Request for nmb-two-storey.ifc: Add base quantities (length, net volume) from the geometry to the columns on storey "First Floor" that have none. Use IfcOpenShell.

First a look at what the model holds.

```python
import ifcopenshell
import ifcopenshell.util.element
import ifcopenshell.util.unit

model = ifcopenshell.open("nmb-two-storey.ifc")
print(model.schema)
for unit_type in ("LENGTHUNIT", "AREAUNIT", "VOLUMEUNIT"):
    print(unit_type, ifcopenshell.util.unit.calculate_unit_scale(model, unit_type))
storey = next(s for s in model.by_type("IfcBuildingStorey") if s.Name == "First Floor")
columns = [e for e in ifcopenshell.util.element.get_decomposition(storey) if e.is_a("IfcColumn")]
for e in sorted(columns, key=lambda e: e.id()):
    print(e.id(), e.is_a(), e.Name, list(ifcopenshell.util.element.get_psets(e, qtos_only=True)), sep=" | ")
```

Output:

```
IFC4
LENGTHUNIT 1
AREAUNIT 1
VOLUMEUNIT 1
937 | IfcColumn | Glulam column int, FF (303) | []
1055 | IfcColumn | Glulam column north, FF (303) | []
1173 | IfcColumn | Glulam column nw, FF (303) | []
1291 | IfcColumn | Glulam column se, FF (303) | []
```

```python
import ifcopenshell
import ifcopenshell.api.pset
import ifcopenshell.geom
import ifcopenshell.util.element
import ifcopenshell.util.shape
import ifcopenshell.util.unit

model = ifcopenshell.open("nmb-two-storey.ifc")
unit_scale = ifcopenshell.util.unit.calculate_unit_scale(model)
volume_scale = ifcopenshell.util.unit.calculate_unit_scale(model, "VOLUMEUNIT")
settings = ifcopenshell.geom.settings()

storey = next(s for s in model.by_type("IfcBuildingStorey") if s.Name == "First Floor")
columns = [e for e in ifcopenshell.util.element.get_decomposition(storey) if e.is_a("IfcColumn")]

for e in sorted(columns, key=lambda e: e.id()):
    if ifcopenshell.util.element.get_psets(e, qtos_only=True, should_inherit=False):
        continue
    # Geometry comes back in metres, in the element's own axes.
    shape = ifcopenshell.geom.create_shape(settings, e)
    values = {
        "Length": ifcopenshell.util.shape.get_z(shape.geometry) / unit_scale,
        "NetVolume": ifcopenshell.util.shape.get_volume(shape.geometry) / volume_scale,
    }
    qto = ifcopenshell.api.pset.add_qto(model, product=e, name="Qto_ColumnBaseQuantities")
    ifcopenshell.api.pset.edit_qto(model, qto=qto, properties=values)
    print(e.id(), {k: round(v, 3) for k, v in values.items()})

model.write("nmb-two-storey_rev.ifc")
```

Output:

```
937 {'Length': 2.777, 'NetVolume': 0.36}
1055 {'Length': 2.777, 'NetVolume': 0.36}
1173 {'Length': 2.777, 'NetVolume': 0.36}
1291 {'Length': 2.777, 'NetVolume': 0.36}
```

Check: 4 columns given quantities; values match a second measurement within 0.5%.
